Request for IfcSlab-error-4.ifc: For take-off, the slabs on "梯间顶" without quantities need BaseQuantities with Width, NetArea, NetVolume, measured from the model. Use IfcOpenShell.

First a look at what the model holds.

```python
import ifcopenshell
import ifcopenshell.util.element
import ifcopenshell.util.unit

model = ifcopenshell.open("IfcSlab-error-4.ifc")
print(model.schema)
for unit_type in ("LENGTHUNIT", "AREAUNIT", "VOLUMEUNIT"):
    print(unit_type, ifcopenshell.util.unit.calculate_unit_scale(model, unit_type))
storey = next(s for s in model.by_type("IfcBuildingStorey") if s.Name == "梯间顶")
slabs = [e for e in ifcopenshell.util.element.get_decomposition(storey) if e.is_a("IfcSlab")]
for e in sorted(slabs, key=lambda e: e.id()):
    print(e.id(), e.is_a(), e.Name, list(ifcopenshell.util.element.get_psets(e, qtos_only=True)), sep=" | ")
```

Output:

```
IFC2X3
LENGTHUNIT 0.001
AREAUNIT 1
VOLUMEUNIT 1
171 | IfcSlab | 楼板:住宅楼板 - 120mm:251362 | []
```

```python
import ifcopenshell
import ifcopenshell.api.pset
import ifcopenshell.geom
import ifcopenshell.util.element
import ifcopenshell.util.shape
import ifcopenshell.util.unit

model = ifcopenshell.open("IfcSlab-error-4.ifc")
unit_scale = ifcopenshell.util.unit.calculate_unit_scale(model)
area_scale = ifcopenshell.util.unit.calculate_unit_scale(model, "AREAUNIT")
volume_scale = ifcopenshell.util.unit.calculate_unit_scale(model, "VOLUMEUNIT")
settings = ifcopenshell.geom.settings()

storey = next(s for s in model.by_type("IfcBuildingStorey") if s.Name == "梯间顶")
slabs = [e for e in ifcopenshell.util.element.get_decomposition(storey) if e.is_a("IfcSlab")]

for e in sorted(slabs, key=lambda e: e.id()):
    if ifcopenshell.util.element.get_psets(e, qtos_only=True, should_inherit=False):
        continue
    # Geometry comes back in metres, in the element's own axes.
    shape = ifcopenshell.geom.create_shape(settings, e)
    values = {
        "Width": ifcopenshell.util.shape.get_z(shape.geometry) / unit_scale,
        "NetArea": ifcopenshell.util.shape.get_footprint_area(shape.geometry) / area_scale,
        "NetVolume": ifcopenshell.util.shape.get_volume(shape.geometry) / volume_scale,
    }
    qto = ifcopenshell.api.pset.add_qto(model, product=e, name="BaseQuantities")
    ifcopenshell.api.pset.edit_qto(model, qto=qto, properties=values)
    print(e.id(), {k: round(v, 3) for k, v in values.items()})

model.write("IfcSlab-error-4_v2.ifc")
```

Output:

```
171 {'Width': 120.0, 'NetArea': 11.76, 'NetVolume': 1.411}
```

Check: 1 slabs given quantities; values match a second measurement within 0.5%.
